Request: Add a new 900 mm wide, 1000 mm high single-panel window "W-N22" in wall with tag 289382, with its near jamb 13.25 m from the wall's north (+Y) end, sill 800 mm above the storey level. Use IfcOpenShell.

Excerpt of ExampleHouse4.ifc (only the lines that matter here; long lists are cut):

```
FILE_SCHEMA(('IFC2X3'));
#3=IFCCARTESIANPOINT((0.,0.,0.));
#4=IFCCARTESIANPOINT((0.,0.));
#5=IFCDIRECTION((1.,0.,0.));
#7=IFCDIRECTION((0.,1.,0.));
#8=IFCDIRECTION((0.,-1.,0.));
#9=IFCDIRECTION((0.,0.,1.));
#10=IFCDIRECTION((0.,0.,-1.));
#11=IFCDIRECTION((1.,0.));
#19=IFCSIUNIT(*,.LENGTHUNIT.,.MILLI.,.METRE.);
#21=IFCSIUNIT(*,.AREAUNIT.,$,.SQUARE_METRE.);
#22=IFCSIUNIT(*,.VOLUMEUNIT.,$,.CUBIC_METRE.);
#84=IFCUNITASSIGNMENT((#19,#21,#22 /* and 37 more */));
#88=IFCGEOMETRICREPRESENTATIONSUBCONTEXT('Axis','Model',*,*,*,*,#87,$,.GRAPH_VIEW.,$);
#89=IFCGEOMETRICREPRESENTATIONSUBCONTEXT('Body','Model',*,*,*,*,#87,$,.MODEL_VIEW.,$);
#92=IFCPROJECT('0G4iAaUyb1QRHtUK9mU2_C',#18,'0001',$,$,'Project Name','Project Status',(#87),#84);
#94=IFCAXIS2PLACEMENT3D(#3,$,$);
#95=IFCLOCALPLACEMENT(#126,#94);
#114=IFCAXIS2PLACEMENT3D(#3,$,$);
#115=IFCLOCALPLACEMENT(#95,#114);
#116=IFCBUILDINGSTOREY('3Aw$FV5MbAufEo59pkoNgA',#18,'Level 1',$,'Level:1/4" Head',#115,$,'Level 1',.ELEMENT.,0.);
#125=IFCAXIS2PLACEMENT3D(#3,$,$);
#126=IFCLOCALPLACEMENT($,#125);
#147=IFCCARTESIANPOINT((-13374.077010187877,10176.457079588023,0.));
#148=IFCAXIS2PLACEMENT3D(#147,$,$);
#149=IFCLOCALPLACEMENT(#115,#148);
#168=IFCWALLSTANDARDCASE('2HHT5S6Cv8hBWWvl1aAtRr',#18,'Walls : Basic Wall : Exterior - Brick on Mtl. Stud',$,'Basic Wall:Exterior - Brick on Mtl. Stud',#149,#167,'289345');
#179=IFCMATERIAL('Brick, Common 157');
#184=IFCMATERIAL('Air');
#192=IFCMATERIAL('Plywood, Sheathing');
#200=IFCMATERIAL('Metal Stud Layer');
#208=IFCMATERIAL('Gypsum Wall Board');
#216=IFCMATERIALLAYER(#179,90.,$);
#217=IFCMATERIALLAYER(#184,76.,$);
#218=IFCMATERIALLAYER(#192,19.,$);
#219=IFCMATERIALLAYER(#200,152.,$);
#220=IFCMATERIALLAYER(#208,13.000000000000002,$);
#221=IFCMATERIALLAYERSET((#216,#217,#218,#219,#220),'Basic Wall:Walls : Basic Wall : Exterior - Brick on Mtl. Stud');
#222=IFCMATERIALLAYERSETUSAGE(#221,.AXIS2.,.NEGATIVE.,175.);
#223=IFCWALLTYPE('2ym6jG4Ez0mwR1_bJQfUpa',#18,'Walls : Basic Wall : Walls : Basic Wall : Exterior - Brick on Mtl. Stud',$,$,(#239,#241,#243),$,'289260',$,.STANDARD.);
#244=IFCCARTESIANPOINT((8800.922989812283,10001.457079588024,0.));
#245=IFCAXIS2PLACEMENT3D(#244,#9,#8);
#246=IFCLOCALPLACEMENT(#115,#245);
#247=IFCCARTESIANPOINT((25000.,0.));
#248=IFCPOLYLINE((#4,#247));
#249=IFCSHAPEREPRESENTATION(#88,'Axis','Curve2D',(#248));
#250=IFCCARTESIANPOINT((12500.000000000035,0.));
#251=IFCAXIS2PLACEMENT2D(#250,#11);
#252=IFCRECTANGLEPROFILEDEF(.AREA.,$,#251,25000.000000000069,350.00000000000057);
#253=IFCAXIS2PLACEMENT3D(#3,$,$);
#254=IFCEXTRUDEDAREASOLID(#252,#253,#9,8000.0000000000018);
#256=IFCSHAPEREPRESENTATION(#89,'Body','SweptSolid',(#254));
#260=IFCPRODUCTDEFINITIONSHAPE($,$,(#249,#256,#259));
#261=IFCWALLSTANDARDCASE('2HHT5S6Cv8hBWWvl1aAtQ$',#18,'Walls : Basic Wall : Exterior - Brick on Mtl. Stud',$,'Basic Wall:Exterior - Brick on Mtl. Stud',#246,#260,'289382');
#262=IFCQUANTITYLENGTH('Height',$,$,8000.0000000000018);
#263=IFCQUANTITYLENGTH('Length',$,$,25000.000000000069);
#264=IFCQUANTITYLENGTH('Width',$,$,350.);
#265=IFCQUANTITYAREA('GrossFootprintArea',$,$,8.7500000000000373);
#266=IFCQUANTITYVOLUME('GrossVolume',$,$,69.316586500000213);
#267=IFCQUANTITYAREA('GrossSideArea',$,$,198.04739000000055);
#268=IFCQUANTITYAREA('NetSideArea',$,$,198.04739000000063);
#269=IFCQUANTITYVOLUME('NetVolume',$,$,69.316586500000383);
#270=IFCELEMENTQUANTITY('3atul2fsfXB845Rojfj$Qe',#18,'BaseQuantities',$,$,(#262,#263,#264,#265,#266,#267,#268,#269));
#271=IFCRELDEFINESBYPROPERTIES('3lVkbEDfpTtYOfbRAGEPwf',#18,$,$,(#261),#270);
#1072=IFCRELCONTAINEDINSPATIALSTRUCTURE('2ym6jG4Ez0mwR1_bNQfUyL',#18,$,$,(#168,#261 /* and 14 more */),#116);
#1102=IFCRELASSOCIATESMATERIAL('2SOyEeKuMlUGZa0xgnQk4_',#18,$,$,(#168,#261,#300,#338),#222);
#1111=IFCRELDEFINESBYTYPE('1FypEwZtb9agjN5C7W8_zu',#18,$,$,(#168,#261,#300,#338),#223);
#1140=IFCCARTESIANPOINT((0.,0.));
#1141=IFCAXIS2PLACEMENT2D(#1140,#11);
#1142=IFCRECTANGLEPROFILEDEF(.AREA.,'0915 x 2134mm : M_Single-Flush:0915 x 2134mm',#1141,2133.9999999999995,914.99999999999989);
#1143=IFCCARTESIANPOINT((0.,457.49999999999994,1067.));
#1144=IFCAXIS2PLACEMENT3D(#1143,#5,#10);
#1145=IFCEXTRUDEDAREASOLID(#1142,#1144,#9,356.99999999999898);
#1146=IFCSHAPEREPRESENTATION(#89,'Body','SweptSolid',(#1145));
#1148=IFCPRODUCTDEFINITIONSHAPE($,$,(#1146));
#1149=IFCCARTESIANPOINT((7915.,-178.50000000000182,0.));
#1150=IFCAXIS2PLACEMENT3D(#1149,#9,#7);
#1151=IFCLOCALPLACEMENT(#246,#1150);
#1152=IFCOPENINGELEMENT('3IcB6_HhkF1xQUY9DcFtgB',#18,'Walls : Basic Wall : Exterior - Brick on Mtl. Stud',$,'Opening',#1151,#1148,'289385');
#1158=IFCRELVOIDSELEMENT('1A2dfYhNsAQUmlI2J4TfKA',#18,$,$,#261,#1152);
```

```python
import numpy as np
import ifcopenshell
import ifcopenshell.api.feature
import ifcopenshell.api.geometry
import ifcopenshell.api.pset
import ifcopenshell.api.root
import ifcopenshell.api.spatial
import ifcopenshell.api.type
import ifcopenshell.geom
import ifcopenshell.util.element
import ifcopenshell.util.placement
import ifcopenshell.util.representation
import ifcopenshell.util.shape
import ifcopenshell.util.unit

model = ifcopenshell.open("ExampleHouse4.ifc")
unit_scale = ifcopenshell.util.unit.calculate_unit_scale(model)
area_scale = ifcopenshell.util.unit.calculate_unit_scale(model, "AREAUNIT")
volume_scale = ifcopenshell.util.unit.calculate_unit_scale(model, "VOLUMEUNIT")
settings = ifcopenshell.geom.settings()


def volume(element):
    """Net volume in cubic metres, openings subtracted."""
    shape = ifcopenshell.geom.create_shape(settings, element)
    return ifcopenshell.util.shape.get_volume(shape.geometry)


wall = model.by_id(261)
storey = ifcopenshell.util.element.get_container(wall, ifc_class="IfcBuildingStorey")
context = ifcopenshell.util.representation.get_context(model, "Model", "Body", "MODEL_VIEW")
before = volume(wall)

width, height, from_end, sill = 0.9, 1, 13.25, 0.8  # metres

# The wall runs along its own X axis, and the end named is its -X end.
wall_shape = ifcopenshell.geom.create_shape(settings, wall)
x, y, z = ifcopenshell.util.shape.get_vertices(wall_shape.geometry).T
start = x.min() + from_end
face, thickness = float(y.min()), float(y.max() - y.min())
wall_matrix = ifcopenshell.util.placement.get_local_placement(wall.ObjectPlacement)
level = ifcopenshell.util.placement.get_local_placement(storey.ObjectPlacement)[2, 3]


def in_wall(x, y):
    """Placement at x, y metres in the wall's axes, at sill height."""
    matrix = wall_matrix.copy()
    matrix[:, 3] = wall_matrix @ np.array([x / unit_scale, y / unit_scale, 0.0, 1.0])
    matrix[2, 3] = level + sill / unit_scale
    return matrix


# Opening: a box that overshoots both wall faces by 50 mm.
opening = ifcopenshell.api.root.create_entity(model, ifc_class="IfcOpeningElement")
box = ifcopenshell.api.geometry.add_wall_representation(
    model, context=context, length=width, height=height, thickness=thickness + 0.1
)
ifcopenshell.api.geometry.assign_representation(model, product=opening, representation=box)
ifcopenshell.api.geometry.edit_object_placement(model, product=opening, matrix=in_wall(start, face - 0.05), is_si=False)
ifcopenshell.api.feature.add_feature(model, feature=opening, element=wall)

window = ifcopenshell.api.root.create_entity(model, ifc_class="IfcWindow", name="W-N22")
window.OverallWidth, window.OverallHeight = width / unit_scale, height / unit_scale
body = ifcopenshell.api.geometry.add_window_representation(
    model,
    context=context,
    overall_width=window.OverallWidth,
    overall_height=window.OverallHeight,
    partition_type="SINGLE_PANEL",
)
ifcopenshell.api.geometry.assign_representation(model, product=window, representation=body)
ifcopenshell.api.spatial.assign_container(model, products=[window], relating_structure=storey)
fills = ifcopenshell.api.feature.add_filling(model, opening=opening, element=window)
fills.OwnerHistory = window.OwnerHistory  # required in IFC2X3

# IFC2X3 keeps the operation on the window style.
style = ifcopenshell.api.root.create_entity(model, ifc_class="IfcWindowStyle", name="W-N22")
style.OperationType, style.ConstructionType = "SINGLE_PANEL", "NOTDEFINED"
style.ParameterTakesPrecedence = style.Sizeable = False
ifcopenshell.api.type.assign_type(model, related_objects=[window], relating_type=style)

# Centre the window in the wall's thickness.
ifcopenshell.api.geometry.edit_object_placement(model, product=window, matrix=in_wall(start, face), is_si=False)
window_shape = ifcopenshell.geom.create_shape(settings, window)
depth = ifcopenshell.util.shape.get_vertices(window_shape.geometry)[:, 1]
offset = face + thickness / 2 - (depth.min() + depth.max()) / 2
ifcopenshell.api.geometry.edit_object_placement(model, product=window, matrix=in_wall(start, offset), is_si=False)

after = volume(wall)

# Update the wall's stored quantities.
qto = model.by_id(ifcopenshell.util.element.get_pset(wall, "BaseQuantities", should_inherit=False)["id"])
ifcopenshell.api.pset.edit_qto(model, qto=qto, properties={
    "NetSideArea": after / thickness / area_scale,
    "NetVolume": after / volume_scale,
})

print(f"wall volume {before:.3f} -> {after:.3f} m3")

model.write("ExampleHouse4_rev.ifc")
```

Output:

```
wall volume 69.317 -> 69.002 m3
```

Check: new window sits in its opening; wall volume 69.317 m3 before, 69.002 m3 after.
